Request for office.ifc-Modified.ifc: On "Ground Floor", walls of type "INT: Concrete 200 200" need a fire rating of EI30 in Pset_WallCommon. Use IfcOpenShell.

First a look at what the model holds.

```python
import ifcopenshell
import ifcopenshell.util.element

model = ifcopenshell.open("office.ifc-Modified.ifc")
print(model.schema)
storey = next(s for s in model.by_type("IfcBuildingStorey") if s.Name == "Ground Floor")
walls = [e for e in ifcopenshell.util.element.get_decomposition(storey) if e.is_a("IfcWall")]
seen = {}
for e in walls:
    element_type = ifcopenshell.util.element.get_type(e)
    key = (element_type.Name if element_type != e and element_type else None, ifcopenshell.util.element.get_pset(e, "Pset_WallCommon", "FireRating"))
    seen[key] = seen.get(key, 0) + 1
for (name, value), count in sorted(seen.items(), key=str):
    print(count, "x", name, "|", value)
```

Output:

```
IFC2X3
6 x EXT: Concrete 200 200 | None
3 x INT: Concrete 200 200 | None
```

```python
import ifcopenshell
import ifcopenshell.api.pset
import ifcopenshell.util.element

model = ifcopenshell.open("office.ifc-Modified.ifc")

storey = next(s for s in model.by_type("IfcBuildingStorey") if s.Name == "Ground Floor")
walls = [e for e in ifcopenshell.util.element.get_decomposition(storey) if e.is_a("IfcWall")]

count = 0
for e in walls:
    element_type = ifcopenshell.util.element.get_type(e)
    if element_type in (None, e) or element_type.Name != "INT: Concrete 200 200":
        continue
    # add_pset returns the element's existing set when there is one.
    pset = ifcopenshell.api.pset.add_pset(model, product=e, name="Pset_WallCommon")
    ifcopenshell.api.pset.edit_pset(model, pset=pset, properties={"FireRating": "EI30"})
    count += 1

print(count, "walls updated")

model.write("office.ifc-Modified-out.ifc")
```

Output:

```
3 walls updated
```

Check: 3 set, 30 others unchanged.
